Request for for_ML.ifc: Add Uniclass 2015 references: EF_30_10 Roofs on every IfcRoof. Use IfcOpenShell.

First a look at what the model holds.

```python
import ifcopenshell

model = ifcopenshell.open("for_ML.ifc")
print(model.schema)
print("classifications:", [c.Name for c in model.by_type("IfcClassification")])
for ifc_class in ("IfcDoor", "IfcRoof", "IfcStair", "IfcWall", "IfcWindow"):
    print(ifc_class, len(model.by_type(ifc_class)))
```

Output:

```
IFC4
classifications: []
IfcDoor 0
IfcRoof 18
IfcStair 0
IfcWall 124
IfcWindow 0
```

```python
import ifcopenshell
import ifcopenshell.api.classification

model = ifcopenshell.open("for_ML.ifc")

system = ifcopenshell.api.classification.add_classification(model, classification="Uniclass 2015")

codes = {
    "IfcRoof": ("EF_30_10", "Roofs"),
}
for ifc_class, (code, name) in codes.items():
    products = model.by_type(ifc_class)
    ifcopenshell.api.classification.add_reference(
        model, products=products, classification=system, identification=code, name=name
    )
    print(code, len(products))

model.write("for_ML-out.ifc")
```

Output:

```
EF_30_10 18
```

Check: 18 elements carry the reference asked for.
